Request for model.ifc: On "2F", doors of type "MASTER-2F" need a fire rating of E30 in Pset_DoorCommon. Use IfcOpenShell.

First a look at what the model holds.

```python
import ifcopenshell
import ifcopenshell.util.element

model = ifcopenshell.open("model.ifc")
print(model.schema)
storey = next(s for s in model.by_type("IfcBuildingStorey") if s.Name == "2F")
doors = [e for e in ifcopenshell.util.element.get_decomposition(storey) if e.is_a("IfcDoor")]
seen = {}
for e in doors:
    element_type = ifcopenshell.util.element.get_type(e)
    key = (element_type.Name if element_type != e and element_type else None, ifcopenshell.util.element.get_pset(e, "Pset_DoorCommon", "FireRating"))
    seen[key] = seen.get(key, 0) + 1
for (name, value), count in sorted(seen.items(), key=str):
    print(count, "x", name, "|", value)
```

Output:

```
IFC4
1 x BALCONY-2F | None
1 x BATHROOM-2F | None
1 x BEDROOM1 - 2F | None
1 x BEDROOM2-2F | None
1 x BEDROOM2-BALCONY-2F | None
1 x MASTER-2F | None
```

```python
import ifcopenshell
import ifcopenshell.api.pset
import ifcopenshell.util.element

model = ifcopenshell.open("model.ifc")

storey = next(s for s in model.by_type("IfcBuildingStorey") if s.Name == "2F")
doors = [e for e in ifcopenshell.util.element.get_decomposition(storey) if e.is_a("IfcDoor")]

count = 0
for e in doors:
    element_type = ifcopenshell.util.element.get_type(e)
    if element_type in (None, e) or element_type.Name != "MASTER-2F":
        continue
    # add_pset returns the element's existing set when there is one.
    pset = ifcopenshell.api.pset.add_pset(model, product=e, name="Pset_DoorCommon")
    ifcopenshell.api.pset.edit_pset(model, pset=pset, properties={"FireRating": "E30"})
    count += 1

print(count, "doors updated")

model.write("model_rev.ifc")
```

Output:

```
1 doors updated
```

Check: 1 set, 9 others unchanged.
